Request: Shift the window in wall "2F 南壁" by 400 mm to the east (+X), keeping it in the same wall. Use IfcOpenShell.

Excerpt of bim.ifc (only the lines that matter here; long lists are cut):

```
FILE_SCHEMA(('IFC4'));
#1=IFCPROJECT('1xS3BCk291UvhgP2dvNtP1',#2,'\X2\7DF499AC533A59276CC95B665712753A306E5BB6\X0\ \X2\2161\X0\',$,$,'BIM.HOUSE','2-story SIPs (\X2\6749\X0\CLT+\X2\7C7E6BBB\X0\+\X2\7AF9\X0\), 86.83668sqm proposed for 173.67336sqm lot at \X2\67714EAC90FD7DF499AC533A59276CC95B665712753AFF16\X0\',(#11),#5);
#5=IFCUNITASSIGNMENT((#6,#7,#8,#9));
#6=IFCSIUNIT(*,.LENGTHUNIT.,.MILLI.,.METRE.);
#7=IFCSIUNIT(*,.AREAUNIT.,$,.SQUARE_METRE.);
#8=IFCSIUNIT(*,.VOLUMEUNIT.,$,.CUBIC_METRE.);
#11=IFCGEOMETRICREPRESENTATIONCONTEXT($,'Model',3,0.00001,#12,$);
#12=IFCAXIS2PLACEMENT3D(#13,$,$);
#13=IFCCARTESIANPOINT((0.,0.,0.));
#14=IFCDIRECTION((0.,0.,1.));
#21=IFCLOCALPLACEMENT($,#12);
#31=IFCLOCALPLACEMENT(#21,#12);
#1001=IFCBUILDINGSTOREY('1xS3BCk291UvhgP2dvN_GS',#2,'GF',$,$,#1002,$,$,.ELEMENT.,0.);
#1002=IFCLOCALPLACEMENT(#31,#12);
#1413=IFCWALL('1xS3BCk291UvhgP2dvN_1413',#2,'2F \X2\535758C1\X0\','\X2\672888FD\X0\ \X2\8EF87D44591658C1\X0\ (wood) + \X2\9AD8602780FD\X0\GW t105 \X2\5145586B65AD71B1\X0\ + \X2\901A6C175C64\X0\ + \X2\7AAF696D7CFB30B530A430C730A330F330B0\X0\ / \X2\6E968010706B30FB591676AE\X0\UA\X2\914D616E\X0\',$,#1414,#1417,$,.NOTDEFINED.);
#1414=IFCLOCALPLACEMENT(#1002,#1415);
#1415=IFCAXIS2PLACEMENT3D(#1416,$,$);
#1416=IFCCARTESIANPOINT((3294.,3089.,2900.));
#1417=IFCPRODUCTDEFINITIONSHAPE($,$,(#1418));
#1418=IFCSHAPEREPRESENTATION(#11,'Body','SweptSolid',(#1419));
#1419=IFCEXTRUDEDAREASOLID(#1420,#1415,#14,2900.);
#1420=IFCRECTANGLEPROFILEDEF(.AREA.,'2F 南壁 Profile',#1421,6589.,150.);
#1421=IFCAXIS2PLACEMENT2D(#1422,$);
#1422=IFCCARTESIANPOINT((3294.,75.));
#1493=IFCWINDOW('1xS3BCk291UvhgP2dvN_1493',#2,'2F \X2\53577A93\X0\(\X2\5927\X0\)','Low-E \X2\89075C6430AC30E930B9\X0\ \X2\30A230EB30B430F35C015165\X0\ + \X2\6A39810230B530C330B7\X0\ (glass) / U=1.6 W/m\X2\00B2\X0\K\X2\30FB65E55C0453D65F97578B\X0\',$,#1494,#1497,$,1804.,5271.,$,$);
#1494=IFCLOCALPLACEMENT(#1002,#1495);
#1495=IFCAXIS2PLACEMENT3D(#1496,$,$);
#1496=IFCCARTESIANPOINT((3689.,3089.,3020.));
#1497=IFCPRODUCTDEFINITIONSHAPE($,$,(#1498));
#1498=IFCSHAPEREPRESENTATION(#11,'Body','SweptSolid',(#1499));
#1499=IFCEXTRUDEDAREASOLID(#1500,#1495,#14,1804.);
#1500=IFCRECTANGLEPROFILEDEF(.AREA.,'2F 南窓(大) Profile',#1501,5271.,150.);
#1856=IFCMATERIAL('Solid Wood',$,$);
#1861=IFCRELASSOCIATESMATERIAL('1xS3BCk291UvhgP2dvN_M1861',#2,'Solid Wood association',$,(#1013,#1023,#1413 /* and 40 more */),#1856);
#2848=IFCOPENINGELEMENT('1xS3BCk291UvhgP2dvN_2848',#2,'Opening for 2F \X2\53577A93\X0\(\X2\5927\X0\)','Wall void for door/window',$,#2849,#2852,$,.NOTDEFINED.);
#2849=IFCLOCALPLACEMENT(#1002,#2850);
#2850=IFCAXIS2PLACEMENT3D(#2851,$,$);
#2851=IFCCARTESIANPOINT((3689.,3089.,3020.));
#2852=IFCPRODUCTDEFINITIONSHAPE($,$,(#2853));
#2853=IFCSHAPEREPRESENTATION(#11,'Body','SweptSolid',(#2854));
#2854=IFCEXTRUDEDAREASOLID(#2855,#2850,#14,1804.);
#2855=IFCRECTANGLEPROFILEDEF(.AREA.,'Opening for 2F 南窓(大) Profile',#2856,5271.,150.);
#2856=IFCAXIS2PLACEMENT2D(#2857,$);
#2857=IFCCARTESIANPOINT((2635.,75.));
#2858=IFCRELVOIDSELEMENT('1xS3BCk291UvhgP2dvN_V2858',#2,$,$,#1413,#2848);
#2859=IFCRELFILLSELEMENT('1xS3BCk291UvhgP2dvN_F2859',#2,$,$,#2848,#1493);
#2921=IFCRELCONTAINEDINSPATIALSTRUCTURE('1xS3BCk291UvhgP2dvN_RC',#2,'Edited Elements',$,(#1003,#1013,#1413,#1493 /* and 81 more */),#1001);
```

```python
import ifcopenshell
import ifcopenshell.api.geometry
import ifcopenshell.util.placement
import ifcopenshell.util.unit

model = ifcopenshell.open("bim.ifc")
unit_scale = ifcopenshell.util.unit.calculate_unit_scale(model)

window = model.by_guid("1xS3BCk291UvhgP2dvN_1493")
opening = window.FillsVoids[0].RelatingOpeningElement
wall = opening.VoidsElements[0].RelatingBuildingElement

wall_matrix = ifcopenshell.util.placement.get_local_placement(wall.ObjectPlacement)
shift = wall_matrix[:3, 0] * 0.4 / unit_scale
before = ifcopenshell.util.placement.get_local_placement(window.ObjectPlacement)[:3, 3].copy()

# The window is not placed relative to its opening, so move both.
for product in (opening, window):
    matrix = ifcopenshell.util.placement.get_local_placement(product.ObjectPlacement)
    matrix[:3, 3] += shift
    ifcopenshell.api.geometry.edit_object_placement(model, product=product, matrix=matrix, is_si=False)

after = ifcopenshell.util.placement.get_local_placement(window.ObjectPlacement)[:3, 3]
print("window moved by", (after - before).round(3) + 0.0)

model.write("bim_updated.ifc")
```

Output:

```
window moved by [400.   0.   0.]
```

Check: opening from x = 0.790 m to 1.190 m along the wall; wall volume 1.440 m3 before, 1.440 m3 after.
